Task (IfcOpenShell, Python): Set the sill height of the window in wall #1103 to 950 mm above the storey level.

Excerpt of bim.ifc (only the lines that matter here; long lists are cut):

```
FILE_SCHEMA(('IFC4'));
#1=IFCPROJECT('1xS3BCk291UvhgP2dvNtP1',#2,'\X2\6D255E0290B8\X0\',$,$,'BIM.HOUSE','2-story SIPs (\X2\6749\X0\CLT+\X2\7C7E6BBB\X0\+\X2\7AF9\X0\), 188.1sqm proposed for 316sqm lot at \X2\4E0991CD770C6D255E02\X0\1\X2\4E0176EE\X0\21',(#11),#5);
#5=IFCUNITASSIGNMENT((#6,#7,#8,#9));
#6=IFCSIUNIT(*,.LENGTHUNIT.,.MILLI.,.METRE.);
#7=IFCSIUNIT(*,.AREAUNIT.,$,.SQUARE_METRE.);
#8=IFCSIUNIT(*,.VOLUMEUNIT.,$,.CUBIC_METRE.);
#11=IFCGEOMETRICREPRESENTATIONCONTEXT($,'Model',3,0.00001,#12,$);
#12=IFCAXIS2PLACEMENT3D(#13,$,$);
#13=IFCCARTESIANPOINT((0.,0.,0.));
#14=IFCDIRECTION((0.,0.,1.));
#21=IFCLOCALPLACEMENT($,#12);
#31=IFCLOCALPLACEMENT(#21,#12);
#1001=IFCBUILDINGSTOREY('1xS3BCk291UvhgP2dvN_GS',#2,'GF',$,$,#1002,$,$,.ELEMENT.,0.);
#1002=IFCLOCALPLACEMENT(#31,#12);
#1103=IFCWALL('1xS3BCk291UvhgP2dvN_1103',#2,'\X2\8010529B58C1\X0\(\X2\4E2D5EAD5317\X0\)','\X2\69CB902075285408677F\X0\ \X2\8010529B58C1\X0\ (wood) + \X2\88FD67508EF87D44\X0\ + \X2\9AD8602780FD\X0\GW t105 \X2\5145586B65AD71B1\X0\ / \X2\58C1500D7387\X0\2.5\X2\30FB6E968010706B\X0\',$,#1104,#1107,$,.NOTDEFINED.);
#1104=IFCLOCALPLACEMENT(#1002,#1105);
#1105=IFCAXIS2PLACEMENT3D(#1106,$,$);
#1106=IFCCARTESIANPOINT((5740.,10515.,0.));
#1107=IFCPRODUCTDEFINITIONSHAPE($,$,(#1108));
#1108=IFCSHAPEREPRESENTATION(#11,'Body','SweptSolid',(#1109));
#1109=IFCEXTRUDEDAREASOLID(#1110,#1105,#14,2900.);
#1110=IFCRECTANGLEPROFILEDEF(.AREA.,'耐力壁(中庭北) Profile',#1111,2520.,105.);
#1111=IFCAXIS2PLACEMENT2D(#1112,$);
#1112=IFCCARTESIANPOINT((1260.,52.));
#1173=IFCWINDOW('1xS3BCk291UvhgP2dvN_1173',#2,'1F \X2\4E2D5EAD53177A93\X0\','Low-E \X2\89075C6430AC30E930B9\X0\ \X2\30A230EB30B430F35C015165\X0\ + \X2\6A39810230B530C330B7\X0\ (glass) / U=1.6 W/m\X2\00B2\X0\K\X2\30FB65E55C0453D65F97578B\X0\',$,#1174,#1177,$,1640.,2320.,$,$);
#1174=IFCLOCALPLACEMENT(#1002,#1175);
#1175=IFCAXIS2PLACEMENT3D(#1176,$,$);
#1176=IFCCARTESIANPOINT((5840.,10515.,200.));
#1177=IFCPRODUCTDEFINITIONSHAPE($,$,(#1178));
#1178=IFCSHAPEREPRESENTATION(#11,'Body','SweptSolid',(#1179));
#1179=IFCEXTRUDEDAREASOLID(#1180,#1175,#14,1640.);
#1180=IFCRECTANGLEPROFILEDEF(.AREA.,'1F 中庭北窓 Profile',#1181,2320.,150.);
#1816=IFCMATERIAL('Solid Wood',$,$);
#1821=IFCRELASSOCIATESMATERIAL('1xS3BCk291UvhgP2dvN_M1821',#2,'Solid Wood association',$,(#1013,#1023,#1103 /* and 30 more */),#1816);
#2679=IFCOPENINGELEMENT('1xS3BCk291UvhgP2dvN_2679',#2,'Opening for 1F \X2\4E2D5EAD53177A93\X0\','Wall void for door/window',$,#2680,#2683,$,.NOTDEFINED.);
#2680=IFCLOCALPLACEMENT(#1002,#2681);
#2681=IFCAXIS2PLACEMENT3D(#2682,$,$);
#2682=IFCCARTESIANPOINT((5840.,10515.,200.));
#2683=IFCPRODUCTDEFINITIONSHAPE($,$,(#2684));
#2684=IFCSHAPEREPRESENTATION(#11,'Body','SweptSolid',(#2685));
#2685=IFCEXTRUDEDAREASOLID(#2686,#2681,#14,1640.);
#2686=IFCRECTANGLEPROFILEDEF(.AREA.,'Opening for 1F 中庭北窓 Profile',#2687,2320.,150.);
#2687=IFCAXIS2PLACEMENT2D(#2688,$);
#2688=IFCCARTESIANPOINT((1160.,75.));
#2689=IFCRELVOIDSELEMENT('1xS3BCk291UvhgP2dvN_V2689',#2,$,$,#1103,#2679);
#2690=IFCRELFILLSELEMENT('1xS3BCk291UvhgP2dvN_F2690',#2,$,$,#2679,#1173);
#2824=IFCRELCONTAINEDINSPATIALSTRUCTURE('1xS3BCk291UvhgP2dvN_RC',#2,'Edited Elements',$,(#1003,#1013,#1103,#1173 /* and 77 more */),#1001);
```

```python
import numpy as np
import ifcopenshell
import ifcopenshell.api.geometry
import ifcopenshell.geom
import ifcopenshell.util.element
import ifcopenshell.util.placement
import ifcopenshell.util.shape
import ifcopenshell.util.unit

model = ifcopenshell.open("bim.ifc")
unit_scale = ifcopenshell.util.unit.calculate_unit_scale(model)

window = model.by_guid("1xS3BCk291UvhgP2dvN_1173")
opening = window.FillsVoids[0].RelatingOpeningElement
storey = ifcopenshell.util.element.get_container(window, ifc_class="IfcBuildingStorey")
level = ifcopenshell.util.placement.get_local_placement(storey.ObjectPlacement)[2, 3]

# The opening's origin need not be at the sill, so measure its lowest point.
shape = ifcopenshell.geom.create_shape(ifcopenshell.geom.settings(), opening)
bottom = ifcopenshell.util.shape.get_shape_bottom_elevation(shape, shape.geometry) / unit_scale
dz = level + 0.95 / unit_scale - bottom

shift = np.array([0.0, 0.0, dz])
# The window is not placed relative to its opening, so move both.
for product in (opening, window):
    matrix = ifcopenshell.util.placement.get_local_placement(product.ObjectPlacement)
    matrix[:3, 3] += shift
    ifcopenshell.api.geometry.edit_object_placement(model, product=product, matrix=matrix, is_si=False)

print(f"moved by {dz * unit_scale:+.3f} m")

model.write("bim-out.ifc")
```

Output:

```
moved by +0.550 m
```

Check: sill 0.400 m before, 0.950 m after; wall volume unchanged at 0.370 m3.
